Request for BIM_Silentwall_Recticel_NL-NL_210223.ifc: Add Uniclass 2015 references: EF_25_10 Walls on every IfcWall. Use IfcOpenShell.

First a look at what the model holds.

```python
import ifcopenshell

model = ifcopenshell.open("BIM_Silentwall_Recticel_NL-NL_210223.ifc")
print(model.schema)
print("classifications:", [c.Name for c in model.by_type("IfcClassification")])
for ifc_class in ("IfcDoor", "IfcRoof", "IfcStair", "IfcWall", "IfcWindow"):
    print(ifc_class, len(model.by_type(ifc_class)))
```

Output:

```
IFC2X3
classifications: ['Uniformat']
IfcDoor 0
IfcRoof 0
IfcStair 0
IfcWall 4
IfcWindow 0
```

```python
import ifcopenshell
import ifcopenshell.api.classification

model = ifcopenshell.open("BIM_Silentwall_Recticel_NL-NL_210223.ifc")

# IFC2X3 requires Source and Edition and has no link from the project to the system.
system = model.create_entity("IfcClassification", Source="NBS", Edition="2015", Name="Uniclass 2015")

codes = {
    "IfcWall": ("EF_25_10", "Walls"),
}
for ifc_class, (code, name) in codes.items():
    products = model.by_type(ifc_class)
    ifcopenshell.api.classification.add_reference(
        model, products=products, classification=system, identification=code, name=name
    )
    print(code, len(products))

model.write("BIM_Silentwall_Recticel_NL-NL_210223_rev.ifc")
```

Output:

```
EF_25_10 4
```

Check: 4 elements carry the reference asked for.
